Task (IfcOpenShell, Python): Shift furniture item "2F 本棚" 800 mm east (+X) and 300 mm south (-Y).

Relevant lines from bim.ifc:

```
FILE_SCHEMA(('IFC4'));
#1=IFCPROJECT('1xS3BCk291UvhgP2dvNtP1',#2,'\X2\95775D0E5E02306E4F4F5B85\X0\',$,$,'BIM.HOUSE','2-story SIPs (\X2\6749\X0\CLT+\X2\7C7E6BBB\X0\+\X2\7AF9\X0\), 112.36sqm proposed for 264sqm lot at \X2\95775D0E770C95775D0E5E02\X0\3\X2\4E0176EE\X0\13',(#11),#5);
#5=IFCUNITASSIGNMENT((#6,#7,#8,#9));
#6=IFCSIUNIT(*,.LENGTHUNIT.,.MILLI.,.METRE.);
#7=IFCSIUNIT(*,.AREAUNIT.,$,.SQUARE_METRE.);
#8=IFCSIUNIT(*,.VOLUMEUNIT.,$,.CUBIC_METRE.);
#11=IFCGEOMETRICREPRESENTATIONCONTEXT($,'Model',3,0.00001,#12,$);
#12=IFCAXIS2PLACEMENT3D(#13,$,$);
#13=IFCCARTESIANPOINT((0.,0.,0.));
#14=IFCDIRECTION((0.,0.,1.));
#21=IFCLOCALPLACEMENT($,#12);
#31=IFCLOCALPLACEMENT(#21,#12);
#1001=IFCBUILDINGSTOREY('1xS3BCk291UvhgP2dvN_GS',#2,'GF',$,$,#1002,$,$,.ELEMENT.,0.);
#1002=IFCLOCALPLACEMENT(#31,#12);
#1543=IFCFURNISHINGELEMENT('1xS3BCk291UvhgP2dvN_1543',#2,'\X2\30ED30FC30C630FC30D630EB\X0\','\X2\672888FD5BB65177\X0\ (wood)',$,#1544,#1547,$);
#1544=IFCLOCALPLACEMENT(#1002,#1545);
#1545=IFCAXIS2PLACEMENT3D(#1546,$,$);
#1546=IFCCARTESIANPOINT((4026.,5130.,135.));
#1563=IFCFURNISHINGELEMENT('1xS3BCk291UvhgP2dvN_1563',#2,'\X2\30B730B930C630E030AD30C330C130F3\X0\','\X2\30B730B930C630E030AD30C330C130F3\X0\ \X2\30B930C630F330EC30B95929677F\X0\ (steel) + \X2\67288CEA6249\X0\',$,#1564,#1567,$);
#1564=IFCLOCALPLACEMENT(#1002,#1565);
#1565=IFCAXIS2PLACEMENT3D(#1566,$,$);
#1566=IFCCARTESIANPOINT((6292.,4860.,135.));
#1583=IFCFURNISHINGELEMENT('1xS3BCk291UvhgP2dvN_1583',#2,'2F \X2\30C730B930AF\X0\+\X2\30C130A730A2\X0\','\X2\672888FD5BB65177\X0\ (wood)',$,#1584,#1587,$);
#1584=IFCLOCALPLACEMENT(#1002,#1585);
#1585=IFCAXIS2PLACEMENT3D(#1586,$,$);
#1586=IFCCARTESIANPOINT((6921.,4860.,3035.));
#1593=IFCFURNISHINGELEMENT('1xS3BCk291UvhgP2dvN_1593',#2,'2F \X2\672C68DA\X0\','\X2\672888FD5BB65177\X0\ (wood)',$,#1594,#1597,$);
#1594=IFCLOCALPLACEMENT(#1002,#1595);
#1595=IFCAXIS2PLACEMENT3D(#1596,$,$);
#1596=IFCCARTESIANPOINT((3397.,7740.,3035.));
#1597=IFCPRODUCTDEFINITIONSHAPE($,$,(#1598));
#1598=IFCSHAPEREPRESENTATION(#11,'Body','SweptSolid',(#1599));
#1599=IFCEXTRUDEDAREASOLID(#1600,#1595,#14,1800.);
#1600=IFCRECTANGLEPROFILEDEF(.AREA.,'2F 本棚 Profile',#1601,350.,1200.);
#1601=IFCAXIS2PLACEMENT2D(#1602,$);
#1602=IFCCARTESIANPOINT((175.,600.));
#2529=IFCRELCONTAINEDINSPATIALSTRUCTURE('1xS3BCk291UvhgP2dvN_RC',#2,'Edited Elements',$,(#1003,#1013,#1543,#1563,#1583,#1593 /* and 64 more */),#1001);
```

```python
import ifcopenshell
import ifcopenshell.api.geometry
import ifcopenshell.util.placement
import ifcopenshell.util.unit

model = ifcopenshell.open("bim.ifc")
unit_scale = ifcopenshell.util.unit.calculate_unit_scale(model)

item = model.by_id(1593)
matrix = ifcopenshell.util.placement.get_local_placement(item.ObjectPlacement)
matrix[0, 3] += 0.8 / unit_scale
matrix[1, 3] -= 0.3 / unit_scale
ifcopenshell.api.geometry.edit_object_placement(model, product=item, matrix=matrix, is_si=False)

print(ifcopenshell.util.placement.get_local_placement(item.ObjectPlacement).round(3) + 0.0)

model.write("bim-out.ifc")
```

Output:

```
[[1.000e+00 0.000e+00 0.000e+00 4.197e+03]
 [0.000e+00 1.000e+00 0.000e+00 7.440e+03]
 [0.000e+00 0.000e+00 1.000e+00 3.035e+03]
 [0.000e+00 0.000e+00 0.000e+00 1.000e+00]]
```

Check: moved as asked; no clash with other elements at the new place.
